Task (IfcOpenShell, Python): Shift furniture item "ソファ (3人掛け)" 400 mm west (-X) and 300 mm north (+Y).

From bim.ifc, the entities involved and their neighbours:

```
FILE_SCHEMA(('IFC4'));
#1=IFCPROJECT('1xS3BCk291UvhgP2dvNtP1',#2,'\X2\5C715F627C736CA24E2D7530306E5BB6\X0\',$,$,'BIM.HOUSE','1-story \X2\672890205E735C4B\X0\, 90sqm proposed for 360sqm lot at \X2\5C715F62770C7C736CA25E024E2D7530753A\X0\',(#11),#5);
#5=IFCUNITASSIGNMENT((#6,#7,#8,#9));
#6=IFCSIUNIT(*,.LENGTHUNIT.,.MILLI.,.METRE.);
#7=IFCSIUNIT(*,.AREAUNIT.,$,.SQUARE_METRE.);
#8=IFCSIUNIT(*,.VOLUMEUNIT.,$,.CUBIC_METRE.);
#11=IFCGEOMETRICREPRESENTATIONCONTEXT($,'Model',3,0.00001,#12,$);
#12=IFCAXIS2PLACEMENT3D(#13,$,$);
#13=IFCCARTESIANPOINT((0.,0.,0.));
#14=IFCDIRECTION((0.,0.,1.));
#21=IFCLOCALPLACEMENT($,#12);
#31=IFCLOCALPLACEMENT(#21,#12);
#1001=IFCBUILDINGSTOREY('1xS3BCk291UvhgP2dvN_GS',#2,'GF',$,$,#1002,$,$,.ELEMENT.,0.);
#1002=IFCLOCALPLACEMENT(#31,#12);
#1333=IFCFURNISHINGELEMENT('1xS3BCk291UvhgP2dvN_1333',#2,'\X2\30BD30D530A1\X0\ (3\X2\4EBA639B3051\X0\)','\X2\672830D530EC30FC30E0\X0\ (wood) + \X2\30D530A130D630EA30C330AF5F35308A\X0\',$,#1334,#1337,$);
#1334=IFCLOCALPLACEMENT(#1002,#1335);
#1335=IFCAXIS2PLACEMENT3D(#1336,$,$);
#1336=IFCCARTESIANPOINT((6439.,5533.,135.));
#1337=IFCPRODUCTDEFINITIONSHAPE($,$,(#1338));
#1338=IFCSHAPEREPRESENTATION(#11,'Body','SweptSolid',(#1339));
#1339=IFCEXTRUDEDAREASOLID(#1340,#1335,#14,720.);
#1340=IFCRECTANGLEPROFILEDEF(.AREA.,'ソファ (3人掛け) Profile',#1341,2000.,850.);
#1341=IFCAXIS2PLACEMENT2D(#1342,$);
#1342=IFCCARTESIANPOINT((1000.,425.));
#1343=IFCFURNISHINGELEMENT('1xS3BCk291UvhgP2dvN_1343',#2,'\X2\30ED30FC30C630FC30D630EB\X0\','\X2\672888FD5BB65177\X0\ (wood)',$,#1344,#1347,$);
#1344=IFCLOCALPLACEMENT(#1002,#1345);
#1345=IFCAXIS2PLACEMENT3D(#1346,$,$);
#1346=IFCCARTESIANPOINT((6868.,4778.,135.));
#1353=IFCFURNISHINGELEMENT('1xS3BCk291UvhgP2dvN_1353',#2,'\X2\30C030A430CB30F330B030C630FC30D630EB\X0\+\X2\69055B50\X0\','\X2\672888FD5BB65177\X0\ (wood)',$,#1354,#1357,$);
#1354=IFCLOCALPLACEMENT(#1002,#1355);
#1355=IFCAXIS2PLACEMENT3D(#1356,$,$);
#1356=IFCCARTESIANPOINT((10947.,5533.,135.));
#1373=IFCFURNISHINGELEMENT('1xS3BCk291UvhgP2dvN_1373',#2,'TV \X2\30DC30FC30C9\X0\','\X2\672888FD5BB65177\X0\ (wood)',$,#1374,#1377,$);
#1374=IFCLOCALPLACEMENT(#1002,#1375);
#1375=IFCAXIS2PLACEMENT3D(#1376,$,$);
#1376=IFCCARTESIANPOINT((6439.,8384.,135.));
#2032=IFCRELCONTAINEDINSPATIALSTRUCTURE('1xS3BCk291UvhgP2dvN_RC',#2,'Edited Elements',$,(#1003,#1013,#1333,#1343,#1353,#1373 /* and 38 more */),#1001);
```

```python
import ifcopenshell
import ifcopenshell.api.geometry
import ifcopenshell.util.placement

model = ifcopenshell.open("bim.ifc")

item = model.by_guid("1xS3BCk291UvhgP2dvN_1333")
matrix = ifcopenshell.util.placement.get_local_placement(item.ObjectPlacement)
matrix[0, 3] -= 400.0
matrix[1, 3] += 300.0
ifcopenshell.api.geometry.edit_object_placement(model, product=item, matrix=matrix, is_si=False)

print(ifcopenshell.util.placement.get_local_placement(item.ObjectPlacement).round(3) + 0.0)

model.write("bim_v2.ifc")
```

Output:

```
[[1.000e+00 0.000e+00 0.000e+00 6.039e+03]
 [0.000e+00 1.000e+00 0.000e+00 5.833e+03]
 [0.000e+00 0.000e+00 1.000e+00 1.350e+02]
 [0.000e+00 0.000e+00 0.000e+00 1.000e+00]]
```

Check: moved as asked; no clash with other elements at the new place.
